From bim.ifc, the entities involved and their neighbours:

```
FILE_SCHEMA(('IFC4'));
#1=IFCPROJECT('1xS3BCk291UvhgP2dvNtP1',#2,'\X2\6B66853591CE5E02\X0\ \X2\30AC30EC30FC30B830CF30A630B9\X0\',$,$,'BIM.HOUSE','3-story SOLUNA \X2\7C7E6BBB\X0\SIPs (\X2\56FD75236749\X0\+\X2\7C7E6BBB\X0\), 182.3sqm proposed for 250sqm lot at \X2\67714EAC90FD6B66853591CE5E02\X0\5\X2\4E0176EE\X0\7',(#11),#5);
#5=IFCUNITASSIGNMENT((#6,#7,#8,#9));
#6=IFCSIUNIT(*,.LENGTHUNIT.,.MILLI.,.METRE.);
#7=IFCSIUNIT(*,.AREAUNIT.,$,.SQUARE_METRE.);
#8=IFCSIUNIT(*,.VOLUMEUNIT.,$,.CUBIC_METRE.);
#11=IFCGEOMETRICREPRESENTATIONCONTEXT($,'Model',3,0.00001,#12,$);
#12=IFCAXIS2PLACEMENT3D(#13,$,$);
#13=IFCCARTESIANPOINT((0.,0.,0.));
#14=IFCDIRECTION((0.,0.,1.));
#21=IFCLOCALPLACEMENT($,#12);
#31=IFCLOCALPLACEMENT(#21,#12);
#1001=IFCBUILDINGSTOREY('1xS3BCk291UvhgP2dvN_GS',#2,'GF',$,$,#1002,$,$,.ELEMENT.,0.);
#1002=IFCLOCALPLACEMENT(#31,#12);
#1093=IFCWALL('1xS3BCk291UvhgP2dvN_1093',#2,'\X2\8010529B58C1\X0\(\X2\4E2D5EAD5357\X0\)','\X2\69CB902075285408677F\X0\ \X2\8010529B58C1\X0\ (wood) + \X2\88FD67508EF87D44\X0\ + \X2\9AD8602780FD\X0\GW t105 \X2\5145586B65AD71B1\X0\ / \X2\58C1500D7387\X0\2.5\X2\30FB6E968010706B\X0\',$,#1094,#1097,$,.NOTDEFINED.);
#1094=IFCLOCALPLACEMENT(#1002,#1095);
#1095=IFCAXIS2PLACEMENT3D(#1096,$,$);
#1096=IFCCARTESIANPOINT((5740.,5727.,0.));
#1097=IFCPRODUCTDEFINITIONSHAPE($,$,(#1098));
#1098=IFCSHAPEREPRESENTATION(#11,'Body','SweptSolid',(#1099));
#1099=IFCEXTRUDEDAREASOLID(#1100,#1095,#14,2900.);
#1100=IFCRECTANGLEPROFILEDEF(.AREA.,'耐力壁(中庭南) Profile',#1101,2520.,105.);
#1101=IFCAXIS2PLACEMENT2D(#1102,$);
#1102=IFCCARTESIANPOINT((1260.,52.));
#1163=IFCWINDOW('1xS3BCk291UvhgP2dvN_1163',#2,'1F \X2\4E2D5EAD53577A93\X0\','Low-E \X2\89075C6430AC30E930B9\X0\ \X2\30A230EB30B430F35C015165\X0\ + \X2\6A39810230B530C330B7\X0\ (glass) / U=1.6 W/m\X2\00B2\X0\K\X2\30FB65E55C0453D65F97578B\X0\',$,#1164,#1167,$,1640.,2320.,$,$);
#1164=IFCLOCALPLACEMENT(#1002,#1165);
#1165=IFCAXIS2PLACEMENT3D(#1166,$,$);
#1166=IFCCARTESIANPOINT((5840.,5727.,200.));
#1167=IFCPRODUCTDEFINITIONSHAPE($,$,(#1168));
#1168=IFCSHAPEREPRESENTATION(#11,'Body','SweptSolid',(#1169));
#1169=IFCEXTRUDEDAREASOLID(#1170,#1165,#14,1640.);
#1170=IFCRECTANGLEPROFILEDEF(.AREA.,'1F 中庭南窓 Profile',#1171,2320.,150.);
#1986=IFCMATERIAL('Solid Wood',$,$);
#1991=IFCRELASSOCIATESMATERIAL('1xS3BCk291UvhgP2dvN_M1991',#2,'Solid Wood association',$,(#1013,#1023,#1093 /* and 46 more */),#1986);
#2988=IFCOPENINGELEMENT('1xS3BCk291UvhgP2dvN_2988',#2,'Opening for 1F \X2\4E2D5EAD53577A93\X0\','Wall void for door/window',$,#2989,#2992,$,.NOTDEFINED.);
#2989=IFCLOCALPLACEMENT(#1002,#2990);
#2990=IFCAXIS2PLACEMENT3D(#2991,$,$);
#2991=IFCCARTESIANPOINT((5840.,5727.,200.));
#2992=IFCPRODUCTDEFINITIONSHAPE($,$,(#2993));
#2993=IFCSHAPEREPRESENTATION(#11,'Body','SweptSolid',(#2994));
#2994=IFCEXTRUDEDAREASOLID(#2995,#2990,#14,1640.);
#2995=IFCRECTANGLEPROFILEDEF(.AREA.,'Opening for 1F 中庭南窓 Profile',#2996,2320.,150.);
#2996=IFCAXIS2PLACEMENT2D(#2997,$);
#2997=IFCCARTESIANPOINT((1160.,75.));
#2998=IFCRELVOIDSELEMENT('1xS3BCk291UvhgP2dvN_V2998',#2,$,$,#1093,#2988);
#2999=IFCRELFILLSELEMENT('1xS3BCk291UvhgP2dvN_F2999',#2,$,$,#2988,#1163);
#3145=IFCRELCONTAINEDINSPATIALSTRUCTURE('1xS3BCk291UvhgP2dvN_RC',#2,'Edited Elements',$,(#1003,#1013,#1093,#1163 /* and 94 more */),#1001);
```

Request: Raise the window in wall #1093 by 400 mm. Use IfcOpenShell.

```python
import numpy as np
import ifcopenshell
import ifcopenshell.api.geometry
import ifcopenshell.util.placement
import ifcopenshell.util.unit

model = ifcopenshell.open("bim.ifc")
unit_scale = ifcopenshell.util.unit.calculate_unit_scale(model)

window = model.by_guid("1xS3BCk291UvhgP2dvN_1163")
opening = window.FillsVoids[0].RelatingOpeningElement
dz = 0.4 / unit_scale

shift = np.array([0.0, 0.0, dz])
# The window is not placed relative to its opening, so move both.
for product in (opening, window):
    matrix = ifcopenshell.util.placement.get_local_placement(product.ObjectPlacement)
    matrix[:3, 3] += shift
    ifcopenshell.api.geometry.edit_object_placement(model, product=product, matrix=matrix, is_si=False)

print(f"moved by {dz * unit_scale:+.3f} m")

model.write("bim_updated.ifc")
```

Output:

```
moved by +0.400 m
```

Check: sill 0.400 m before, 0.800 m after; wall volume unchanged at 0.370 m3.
